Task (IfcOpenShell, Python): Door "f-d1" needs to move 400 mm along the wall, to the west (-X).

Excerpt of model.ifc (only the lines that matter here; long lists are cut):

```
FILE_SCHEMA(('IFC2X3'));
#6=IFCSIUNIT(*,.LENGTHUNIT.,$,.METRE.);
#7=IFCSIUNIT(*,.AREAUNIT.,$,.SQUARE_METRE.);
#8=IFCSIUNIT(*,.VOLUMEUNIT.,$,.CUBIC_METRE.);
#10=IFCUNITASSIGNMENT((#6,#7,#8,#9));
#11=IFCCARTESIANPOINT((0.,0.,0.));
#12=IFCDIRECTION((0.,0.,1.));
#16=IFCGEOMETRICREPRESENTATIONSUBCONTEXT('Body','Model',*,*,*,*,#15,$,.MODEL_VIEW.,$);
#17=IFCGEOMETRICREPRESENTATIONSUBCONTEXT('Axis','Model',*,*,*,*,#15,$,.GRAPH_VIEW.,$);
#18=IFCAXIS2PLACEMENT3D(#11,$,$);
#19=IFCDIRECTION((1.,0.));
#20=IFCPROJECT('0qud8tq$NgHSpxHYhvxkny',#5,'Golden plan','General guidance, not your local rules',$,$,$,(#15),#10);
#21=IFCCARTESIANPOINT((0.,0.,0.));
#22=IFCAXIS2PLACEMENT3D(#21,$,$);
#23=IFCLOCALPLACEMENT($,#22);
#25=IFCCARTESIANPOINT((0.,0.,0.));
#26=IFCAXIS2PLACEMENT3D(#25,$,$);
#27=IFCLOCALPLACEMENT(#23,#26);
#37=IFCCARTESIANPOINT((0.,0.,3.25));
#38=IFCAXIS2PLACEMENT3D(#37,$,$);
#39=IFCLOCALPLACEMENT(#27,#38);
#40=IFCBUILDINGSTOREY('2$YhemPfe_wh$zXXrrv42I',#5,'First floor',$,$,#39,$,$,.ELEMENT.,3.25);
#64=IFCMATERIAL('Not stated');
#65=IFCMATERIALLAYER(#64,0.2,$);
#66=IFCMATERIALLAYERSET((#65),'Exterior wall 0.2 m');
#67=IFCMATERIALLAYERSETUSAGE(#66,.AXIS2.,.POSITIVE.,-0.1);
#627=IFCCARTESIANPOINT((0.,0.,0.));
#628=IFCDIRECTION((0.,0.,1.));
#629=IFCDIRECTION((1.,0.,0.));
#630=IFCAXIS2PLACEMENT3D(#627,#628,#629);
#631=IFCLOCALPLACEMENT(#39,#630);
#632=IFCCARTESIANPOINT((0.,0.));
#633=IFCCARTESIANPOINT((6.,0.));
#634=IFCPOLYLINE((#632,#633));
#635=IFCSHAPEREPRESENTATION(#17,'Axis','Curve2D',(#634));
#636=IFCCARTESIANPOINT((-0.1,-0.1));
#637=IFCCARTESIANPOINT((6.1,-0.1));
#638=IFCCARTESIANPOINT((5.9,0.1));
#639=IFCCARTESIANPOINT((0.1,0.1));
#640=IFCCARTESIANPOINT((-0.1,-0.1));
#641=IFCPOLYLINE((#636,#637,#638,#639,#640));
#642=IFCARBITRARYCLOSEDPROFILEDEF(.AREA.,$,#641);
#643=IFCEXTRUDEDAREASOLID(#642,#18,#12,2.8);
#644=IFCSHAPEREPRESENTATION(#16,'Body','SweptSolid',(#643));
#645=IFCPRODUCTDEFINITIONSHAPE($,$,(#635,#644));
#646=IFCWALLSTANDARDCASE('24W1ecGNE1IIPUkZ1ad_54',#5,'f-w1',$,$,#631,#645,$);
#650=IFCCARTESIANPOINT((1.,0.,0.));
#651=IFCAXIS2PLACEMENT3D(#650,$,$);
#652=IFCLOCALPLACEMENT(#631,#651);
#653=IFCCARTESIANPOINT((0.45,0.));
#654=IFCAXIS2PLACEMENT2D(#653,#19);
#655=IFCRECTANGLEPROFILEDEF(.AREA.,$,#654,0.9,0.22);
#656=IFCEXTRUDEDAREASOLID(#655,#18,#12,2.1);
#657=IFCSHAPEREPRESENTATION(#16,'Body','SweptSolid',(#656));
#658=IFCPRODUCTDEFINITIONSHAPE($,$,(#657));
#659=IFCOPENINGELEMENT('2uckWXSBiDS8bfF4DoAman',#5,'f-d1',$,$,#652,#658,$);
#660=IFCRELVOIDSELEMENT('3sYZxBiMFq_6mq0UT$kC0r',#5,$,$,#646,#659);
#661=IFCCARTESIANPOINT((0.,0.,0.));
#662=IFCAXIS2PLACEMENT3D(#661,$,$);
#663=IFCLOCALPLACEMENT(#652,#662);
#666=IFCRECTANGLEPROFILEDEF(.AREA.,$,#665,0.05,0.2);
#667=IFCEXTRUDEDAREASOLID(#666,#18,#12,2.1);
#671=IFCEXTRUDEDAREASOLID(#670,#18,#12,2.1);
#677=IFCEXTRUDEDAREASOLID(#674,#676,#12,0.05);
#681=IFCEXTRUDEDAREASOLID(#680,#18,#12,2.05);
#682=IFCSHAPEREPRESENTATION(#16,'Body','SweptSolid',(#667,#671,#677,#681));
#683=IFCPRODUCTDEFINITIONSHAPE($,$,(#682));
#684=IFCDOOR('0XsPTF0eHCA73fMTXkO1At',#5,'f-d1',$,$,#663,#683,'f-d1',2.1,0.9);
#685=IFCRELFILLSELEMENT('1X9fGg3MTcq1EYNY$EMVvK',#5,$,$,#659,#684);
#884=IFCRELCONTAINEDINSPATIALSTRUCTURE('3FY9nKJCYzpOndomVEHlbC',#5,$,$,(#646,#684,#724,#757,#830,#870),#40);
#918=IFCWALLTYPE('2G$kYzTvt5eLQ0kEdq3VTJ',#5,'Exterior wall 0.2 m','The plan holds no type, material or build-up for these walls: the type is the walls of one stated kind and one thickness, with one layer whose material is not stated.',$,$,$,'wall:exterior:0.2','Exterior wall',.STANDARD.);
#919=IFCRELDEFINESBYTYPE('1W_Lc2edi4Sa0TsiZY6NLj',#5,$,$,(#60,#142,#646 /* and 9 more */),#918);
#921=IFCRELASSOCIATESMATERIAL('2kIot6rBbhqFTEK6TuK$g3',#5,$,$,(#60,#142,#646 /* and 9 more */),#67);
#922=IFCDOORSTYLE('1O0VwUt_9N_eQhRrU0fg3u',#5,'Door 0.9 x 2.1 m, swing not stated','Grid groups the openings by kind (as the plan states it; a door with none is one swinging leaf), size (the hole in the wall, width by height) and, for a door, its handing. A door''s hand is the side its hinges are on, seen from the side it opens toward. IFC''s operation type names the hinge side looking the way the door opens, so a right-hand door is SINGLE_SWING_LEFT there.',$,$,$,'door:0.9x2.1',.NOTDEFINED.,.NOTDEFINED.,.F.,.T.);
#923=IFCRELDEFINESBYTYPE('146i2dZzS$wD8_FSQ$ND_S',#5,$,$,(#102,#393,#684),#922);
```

```python
import ifcopenshell
import ifcopenshell.api.geometry
import ifcopenshell.util.placement
import ifcopenshell.util.unit

model = ifcopenshell.open("model.ifc")
unit_scale = ifcopenshell.util.unit.calculate_unit_scale(model)

door = model.by_guid("0XsPTF0eHCA73fMTXkO1At")
opening = door.FillsVoids[0].RelatingOpeningElement
wall = opening.VoidsElements[0].RelatingBuildingElement

wall_matrix = ifcopenshell.util.placement.get_local_placement(wall.ObjectPlacement)
shift = wall_matrix[:3, 0] * -0.4 / unit_scale
before = ifcopenshell.util.placement.get_local_placement(door.ObjectPlacement)[:3, 3].copy()

# The door is placed relative to its opening, so it follows when the opening moves.
matrix = ifcopenshell.util.placement.get_local_placement(opening.ObjectPlacement)
matrix[:3, 3] += shift
ifcopenshell.api.geometry.edit_object_placement(
    model, product=opening, matrix=matrix, is_si=False, should_transform_children=True
)

after = ifcopenshell.util.placement.get_local_placement(door.ObjectPlacement)[:3, 3]
print("door moved by", (after - before).round(3) + 0.0)

model.write("model_rev.ifc")
```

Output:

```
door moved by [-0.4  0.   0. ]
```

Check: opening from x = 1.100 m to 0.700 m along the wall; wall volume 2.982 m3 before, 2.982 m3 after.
